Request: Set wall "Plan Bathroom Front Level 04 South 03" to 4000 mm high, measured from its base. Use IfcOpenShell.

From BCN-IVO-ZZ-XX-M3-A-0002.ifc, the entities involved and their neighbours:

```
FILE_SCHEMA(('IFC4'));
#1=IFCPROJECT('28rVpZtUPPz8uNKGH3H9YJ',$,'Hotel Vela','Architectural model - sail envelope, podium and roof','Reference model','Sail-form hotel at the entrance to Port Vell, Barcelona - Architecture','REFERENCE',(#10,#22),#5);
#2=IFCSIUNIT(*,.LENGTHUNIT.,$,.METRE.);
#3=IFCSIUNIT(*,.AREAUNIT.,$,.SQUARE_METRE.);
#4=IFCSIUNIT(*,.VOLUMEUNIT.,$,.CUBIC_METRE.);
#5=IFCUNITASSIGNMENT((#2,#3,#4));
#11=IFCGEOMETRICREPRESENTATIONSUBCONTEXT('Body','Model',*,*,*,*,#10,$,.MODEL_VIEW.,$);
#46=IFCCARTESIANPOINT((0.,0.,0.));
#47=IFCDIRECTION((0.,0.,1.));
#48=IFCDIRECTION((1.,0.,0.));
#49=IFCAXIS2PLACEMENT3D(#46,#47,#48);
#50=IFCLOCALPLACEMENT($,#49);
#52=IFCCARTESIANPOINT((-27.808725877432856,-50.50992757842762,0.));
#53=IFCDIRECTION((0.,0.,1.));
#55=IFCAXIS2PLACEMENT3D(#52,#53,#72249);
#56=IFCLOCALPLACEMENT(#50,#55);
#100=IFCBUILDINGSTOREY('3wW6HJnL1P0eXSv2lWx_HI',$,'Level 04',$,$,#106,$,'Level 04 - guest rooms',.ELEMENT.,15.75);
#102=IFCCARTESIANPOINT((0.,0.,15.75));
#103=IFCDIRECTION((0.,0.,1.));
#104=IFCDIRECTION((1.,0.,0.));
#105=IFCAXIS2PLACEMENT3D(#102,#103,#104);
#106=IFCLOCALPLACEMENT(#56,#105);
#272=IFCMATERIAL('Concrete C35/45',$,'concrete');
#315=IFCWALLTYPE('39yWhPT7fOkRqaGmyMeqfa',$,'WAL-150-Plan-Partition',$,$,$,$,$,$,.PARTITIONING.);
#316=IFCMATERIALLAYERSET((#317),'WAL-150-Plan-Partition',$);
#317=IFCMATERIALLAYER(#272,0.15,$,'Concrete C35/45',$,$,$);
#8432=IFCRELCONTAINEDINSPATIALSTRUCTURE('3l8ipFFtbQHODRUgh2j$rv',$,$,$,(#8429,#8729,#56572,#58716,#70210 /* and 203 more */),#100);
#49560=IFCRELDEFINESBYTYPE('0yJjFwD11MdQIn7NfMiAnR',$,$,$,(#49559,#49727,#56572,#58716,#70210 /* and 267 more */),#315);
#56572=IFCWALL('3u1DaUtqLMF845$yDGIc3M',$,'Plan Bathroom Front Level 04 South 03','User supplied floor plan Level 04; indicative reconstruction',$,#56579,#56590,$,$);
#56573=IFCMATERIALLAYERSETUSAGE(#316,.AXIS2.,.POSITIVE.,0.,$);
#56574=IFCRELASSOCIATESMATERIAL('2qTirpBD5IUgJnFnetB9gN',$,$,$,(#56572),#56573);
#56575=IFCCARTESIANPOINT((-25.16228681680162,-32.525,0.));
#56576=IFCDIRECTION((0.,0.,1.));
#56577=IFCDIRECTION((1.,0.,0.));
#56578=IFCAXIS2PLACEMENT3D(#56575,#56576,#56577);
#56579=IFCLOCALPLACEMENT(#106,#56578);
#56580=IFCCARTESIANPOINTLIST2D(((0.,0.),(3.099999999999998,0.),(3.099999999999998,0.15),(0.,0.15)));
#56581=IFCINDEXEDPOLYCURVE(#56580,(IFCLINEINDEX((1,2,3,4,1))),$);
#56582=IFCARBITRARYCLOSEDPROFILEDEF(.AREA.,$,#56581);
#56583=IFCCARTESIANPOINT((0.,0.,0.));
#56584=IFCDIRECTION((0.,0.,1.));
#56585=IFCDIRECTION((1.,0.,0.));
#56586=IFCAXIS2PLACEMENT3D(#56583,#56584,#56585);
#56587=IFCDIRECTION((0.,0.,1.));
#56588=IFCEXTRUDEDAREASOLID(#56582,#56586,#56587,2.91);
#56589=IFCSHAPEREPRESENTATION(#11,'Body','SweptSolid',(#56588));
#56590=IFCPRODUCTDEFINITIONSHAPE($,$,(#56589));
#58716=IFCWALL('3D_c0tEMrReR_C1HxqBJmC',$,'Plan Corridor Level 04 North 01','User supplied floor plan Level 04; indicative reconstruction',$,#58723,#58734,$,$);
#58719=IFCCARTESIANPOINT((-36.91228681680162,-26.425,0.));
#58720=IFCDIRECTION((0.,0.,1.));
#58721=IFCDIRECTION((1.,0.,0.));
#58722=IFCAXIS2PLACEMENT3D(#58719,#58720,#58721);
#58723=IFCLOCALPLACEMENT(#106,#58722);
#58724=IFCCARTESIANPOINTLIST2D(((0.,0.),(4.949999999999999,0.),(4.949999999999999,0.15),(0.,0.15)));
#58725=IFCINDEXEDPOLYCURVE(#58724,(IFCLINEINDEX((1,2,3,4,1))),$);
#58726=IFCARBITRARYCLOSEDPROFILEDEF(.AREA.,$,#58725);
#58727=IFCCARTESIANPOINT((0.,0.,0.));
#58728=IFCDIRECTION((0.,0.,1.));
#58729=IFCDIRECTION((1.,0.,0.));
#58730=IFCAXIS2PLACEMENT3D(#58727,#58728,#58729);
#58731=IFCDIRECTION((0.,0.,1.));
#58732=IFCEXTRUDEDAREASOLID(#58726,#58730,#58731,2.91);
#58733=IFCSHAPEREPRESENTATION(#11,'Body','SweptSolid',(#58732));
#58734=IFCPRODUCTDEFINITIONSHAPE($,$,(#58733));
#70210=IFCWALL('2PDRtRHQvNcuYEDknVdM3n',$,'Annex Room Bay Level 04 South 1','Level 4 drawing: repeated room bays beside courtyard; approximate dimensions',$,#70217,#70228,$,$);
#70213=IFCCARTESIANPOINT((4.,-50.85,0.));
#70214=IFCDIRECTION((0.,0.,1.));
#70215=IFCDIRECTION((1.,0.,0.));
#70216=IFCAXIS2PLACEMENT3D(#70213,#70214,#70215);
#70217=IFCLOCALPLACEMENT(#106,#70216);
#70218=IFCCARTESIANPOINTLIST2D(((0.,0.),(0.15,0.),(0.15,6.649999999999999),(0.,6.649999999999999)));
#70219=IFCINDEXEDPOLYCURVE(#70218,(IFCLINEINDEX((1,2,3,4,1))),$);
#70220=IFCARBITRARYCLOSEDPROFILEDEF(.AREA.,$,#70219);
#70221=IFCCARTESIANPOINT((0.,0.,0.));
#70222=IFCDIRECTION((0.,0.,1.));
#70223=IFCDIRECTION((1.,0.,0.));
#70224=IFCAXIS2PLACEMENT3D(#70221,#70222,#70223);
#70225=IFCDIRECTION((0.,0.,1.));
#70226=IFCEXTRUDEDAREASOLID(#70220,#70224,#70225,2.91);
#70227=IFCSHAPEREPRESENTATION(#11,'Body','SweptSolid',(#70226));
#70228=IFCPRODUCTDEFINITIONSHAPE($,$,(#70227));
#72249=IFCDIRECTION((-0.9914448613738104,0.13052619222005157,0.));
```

```python
import ifcopenshell
import ifcopenshell.geom
import ifcopenshell.util.representation
import ifcopenshell.util.shape
import ifcopenshell.util.unit

model = ifcopenshell.open("BCN-IVO-ZZ-XX-M3-A-0002.ifc")
unit_scale = ifcopenshell.util.unit.calculate_unit_scale(model)
settings = ifcopenshell.geom.settings()


def volume(element):
    """Net volume in cubic metres, openings subtracted."""
    shape = ifcopenshell.geom.create_shape(settings, element)
    return ifcopenshell.util.shape.get_volume(shape.geometry)


wall = model.by_guid("3u1DaUtqLMF845$yDGIc3M")
before = volume(wall)

body = ifcopenshell.util.representation.get_representation(wall, "Model", "Body")
solid = body.Items[0]
old_height = solid.Depth
solid.Depth = 4 / unit_scale
after = volume(wall)

print(f"height {old_height:g} -> {solid.Depth:g}, volume {before:.3f} -> {after:.3f} m3")

model.write("BCN-IVO-ZZ-XX-M3-A-0002_updated.ifc")
```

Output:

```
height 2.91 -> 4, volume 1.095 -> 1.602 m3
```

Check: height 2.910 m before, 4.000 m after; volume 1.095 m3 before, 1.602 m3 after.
